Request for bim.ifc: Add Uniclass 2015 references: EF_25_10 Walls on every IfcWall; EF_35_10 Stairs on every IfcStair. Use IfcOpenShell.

First a look at what the model holds.

```python
import ifcopenshell

model = ifcopenshell.open("bim.ifc")
print(model.schema)
print("classifications:", [c.Name for c in model.by_type("IfcClassification")])
for ifc_class in ("IfcDoor", "IfcRoof", "IfcStair", "IfcWall", "IfcWindow"):
    print(ifc_class, len(model.by_type(ifc_class)))
```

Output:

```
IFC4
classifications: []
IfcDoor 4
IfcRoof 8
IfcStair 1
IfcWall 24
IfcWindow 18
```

```python
import ifcopenshell
import ifcopenshell.api.classification

model = ifcopenshell.open("bim.ifc")

system = ifcopenshell.api.classification.add_classification(model, classification="Uniclass 2015")

codes = {
    "IfcWall": ("EF_25_10", "Walls"),
    "IfcStair": ("EF_35_10", "Stairs"),
}
for ifc_class, (code, name) in codes.items():
    products = model.by_type(ifc_class)
    ifcopenshell.api.classification.add_reference(
        model, products=products, classification=system, identification=code, name=name
    )
    print(code, len(products))

model.write("bim_edited.ifc")
```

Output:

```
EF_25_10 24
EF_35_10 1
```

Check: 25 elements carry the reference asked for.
